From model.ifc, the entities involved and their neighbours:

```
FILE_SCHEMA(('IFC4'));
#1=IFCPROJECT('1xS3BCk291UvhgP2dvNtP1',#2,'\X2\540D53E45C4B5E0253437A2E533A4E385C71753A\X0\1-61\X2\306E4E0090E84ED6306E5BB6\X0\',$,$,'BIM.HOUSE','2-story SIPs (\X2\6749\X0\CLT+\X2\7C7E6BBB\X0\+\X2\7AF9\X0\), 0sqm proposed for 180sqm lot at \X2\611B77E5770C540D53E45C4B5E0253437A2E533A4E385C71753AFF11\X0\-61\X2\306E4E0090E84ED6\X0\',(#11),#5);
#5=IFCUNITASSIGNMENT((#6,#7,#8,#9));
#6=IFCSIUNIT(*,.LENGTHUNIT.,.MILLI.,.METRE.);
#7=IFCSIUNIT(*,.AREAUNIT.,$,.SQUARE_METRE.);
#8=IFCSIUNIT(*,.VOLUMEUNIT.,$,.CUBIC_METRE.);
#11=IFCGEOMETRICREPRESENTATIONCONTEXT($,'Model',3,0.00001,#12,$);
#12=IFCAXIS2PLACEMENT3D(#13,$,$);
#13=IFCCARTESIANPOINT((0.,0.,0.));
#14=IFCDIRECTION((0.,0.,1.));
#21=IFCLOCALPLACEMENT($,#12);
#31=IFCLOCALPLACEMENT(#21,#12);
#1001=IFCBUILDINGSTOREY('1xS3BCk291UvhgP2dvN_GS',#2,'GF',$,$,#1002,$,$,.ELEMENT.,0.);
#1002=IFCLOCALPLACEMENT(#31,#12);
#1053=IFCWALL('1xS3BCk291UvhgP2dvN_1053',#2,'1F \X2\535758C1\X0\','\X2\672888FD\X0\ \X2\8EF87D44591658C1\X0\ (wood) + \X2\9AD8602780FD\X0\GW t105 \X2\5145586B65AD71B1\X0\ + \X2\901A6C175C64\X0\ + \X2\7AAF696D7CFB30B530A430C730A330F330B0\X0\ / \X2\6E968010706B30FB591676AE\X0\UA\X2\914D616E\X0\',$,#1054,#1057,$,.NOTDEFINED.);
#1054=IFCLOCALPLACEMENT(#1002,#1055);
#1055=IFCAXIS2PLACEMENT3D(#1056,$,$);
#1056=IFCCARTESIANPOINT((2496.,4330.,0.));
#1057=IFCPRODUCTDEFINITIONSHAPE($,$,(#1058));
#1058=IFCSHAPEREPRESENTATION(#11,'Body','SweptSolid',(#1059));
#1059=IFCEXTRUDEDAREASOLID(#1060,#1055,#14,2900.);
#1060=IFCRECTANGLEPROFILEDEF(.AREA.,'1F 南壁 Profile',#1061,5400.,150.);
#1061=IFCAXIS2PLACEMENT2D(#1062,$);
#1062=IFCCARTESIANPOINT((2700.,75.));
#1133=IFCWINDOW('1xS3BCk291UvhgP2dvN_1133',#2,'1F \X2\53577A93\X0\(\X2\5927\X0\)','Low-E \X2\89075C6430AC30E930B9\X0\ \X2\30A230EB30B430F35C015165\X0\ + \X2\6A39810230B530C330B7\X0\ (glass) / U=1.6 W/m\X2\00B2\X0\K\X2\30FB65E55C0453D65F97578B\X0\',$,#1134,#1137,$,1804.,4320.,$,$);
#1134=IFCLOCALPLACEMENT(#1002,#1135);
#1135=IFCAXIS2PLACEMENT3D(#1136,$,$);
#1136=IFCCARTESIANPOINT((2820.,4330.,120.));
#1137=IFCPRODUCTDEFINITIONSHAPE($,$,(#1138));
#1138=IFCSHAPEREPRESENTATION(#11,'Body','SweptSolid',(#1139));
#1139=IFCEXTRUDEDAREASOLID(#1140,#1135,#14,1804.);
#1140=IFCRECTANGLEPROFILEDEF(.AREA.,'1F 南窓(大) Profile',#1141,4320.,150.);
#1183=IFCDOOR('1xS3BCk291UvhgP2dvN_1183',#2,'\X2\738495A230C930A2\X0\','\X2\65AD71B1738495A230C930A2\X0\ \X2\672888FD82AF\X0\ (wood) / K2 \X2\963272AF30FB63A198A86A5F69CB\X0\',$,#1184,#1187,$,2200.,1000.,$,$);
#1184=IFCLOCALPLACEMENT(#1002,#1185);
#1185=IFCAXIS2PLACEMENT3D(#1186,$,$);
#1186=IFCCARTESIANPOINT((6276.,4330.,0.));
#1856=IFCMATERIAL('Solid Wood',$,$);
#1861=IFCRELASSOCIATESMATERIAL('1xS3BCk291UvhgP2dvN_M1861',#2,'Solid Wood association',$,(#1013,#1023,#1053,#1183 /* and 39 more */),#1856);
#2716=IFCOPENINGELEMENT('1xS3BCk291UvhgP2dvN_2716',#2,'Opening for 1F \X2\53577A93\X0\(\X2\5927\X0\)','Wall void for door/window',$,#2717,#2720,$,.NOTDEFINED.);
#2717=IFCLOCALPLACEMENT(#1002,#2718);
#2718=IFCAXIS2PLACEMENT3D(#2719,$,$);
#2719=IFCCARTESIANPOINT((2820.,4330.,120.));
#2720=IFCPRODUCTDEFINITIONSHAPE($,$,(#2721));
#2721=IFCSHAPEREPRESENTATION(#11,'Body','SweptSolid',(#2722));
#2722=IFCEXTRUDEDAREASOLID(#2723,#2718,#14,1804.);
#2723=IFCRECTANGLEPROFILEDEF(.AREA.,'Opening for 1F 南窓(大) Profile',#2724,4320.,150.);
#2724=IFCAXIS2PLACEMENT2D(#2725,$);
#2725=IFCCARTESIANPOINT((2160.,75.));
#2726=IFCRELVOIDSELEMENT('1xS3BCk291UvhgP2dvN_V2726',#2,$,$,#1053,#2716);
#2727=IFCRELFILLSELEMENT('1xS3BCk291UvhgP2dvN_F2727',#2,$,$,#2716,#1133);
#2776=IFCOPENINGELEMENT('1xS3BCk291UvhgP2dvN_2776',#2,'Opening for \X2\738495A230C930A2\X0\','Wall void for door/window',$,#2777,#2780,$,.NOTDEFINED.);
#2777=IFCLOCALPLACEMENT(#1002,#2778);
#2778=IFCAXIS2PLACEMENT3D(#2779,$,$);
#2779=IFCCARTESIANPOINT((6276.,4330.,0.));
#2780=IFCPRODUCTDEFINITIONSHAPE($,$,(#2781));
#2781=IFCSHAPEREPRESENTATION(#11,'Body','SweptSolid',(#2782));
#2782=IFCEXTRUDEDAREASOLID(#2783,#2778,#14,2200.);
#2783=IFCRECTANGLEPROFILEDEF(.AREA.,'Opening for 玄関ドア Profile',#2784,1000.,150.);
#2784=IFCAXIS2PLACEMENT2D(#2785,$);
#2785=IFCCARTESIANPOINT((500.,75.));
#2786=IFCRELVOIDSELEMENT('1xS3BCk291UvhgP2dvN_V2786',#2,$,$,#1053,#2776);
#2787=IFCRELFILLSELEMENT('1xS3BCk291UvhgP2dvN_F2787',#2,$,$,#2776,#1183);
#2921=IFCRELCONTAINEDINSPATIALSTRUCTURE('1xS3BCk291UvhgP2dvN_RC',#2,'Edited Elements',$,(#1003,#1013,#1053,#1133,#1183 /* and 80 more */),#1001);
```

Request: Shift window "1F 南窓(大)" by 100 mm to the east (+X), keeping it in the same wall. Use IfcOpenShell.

```python
import ifcopenshell
import ifcopenshell.api.geometry
import ifcopenshell.util.placement

model = ifcopenshell.open("model.ifc")

window = model.by_guid("1xS3BCk291UvhgP2dvN_1133")
opening = window.FillsVoids[0].RelatingOpeningElement
wall = opening.VoidsElements[0].RelatingBuildingElement

wall_matrix = ifcopenshell.util.placement.get_local_placement(wall.ObjectPlacement)
shift = wall_matrix[:3, 0] * 100.0
before = ifcopenshell.util.placement.get_local_placement(window.ObjectPlacement)[:3, 3].copy()

# The window is not placed relative to its opening, so move both.
for product in (opening, window):
    matrix = ifcopenshell.util.placement.get_local_placement(product.ObjectPlacement)
    matrix[:3, 3] += shift
    ifcopenshell.api.geometry.edit_object_placement(model, product=product, matrix=matrix, is_si=False)

after = ifcopenshell.util.placement.get_local_placement(window.ObjectPlacement)[:3, 3]
print("window moved by", (after - before).round(3) + 0.0)

model.write("model_rev.ifc")
```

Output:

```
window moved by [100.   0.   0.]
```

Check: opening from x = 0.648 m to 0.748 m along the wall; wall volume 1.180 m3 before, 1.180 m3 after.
